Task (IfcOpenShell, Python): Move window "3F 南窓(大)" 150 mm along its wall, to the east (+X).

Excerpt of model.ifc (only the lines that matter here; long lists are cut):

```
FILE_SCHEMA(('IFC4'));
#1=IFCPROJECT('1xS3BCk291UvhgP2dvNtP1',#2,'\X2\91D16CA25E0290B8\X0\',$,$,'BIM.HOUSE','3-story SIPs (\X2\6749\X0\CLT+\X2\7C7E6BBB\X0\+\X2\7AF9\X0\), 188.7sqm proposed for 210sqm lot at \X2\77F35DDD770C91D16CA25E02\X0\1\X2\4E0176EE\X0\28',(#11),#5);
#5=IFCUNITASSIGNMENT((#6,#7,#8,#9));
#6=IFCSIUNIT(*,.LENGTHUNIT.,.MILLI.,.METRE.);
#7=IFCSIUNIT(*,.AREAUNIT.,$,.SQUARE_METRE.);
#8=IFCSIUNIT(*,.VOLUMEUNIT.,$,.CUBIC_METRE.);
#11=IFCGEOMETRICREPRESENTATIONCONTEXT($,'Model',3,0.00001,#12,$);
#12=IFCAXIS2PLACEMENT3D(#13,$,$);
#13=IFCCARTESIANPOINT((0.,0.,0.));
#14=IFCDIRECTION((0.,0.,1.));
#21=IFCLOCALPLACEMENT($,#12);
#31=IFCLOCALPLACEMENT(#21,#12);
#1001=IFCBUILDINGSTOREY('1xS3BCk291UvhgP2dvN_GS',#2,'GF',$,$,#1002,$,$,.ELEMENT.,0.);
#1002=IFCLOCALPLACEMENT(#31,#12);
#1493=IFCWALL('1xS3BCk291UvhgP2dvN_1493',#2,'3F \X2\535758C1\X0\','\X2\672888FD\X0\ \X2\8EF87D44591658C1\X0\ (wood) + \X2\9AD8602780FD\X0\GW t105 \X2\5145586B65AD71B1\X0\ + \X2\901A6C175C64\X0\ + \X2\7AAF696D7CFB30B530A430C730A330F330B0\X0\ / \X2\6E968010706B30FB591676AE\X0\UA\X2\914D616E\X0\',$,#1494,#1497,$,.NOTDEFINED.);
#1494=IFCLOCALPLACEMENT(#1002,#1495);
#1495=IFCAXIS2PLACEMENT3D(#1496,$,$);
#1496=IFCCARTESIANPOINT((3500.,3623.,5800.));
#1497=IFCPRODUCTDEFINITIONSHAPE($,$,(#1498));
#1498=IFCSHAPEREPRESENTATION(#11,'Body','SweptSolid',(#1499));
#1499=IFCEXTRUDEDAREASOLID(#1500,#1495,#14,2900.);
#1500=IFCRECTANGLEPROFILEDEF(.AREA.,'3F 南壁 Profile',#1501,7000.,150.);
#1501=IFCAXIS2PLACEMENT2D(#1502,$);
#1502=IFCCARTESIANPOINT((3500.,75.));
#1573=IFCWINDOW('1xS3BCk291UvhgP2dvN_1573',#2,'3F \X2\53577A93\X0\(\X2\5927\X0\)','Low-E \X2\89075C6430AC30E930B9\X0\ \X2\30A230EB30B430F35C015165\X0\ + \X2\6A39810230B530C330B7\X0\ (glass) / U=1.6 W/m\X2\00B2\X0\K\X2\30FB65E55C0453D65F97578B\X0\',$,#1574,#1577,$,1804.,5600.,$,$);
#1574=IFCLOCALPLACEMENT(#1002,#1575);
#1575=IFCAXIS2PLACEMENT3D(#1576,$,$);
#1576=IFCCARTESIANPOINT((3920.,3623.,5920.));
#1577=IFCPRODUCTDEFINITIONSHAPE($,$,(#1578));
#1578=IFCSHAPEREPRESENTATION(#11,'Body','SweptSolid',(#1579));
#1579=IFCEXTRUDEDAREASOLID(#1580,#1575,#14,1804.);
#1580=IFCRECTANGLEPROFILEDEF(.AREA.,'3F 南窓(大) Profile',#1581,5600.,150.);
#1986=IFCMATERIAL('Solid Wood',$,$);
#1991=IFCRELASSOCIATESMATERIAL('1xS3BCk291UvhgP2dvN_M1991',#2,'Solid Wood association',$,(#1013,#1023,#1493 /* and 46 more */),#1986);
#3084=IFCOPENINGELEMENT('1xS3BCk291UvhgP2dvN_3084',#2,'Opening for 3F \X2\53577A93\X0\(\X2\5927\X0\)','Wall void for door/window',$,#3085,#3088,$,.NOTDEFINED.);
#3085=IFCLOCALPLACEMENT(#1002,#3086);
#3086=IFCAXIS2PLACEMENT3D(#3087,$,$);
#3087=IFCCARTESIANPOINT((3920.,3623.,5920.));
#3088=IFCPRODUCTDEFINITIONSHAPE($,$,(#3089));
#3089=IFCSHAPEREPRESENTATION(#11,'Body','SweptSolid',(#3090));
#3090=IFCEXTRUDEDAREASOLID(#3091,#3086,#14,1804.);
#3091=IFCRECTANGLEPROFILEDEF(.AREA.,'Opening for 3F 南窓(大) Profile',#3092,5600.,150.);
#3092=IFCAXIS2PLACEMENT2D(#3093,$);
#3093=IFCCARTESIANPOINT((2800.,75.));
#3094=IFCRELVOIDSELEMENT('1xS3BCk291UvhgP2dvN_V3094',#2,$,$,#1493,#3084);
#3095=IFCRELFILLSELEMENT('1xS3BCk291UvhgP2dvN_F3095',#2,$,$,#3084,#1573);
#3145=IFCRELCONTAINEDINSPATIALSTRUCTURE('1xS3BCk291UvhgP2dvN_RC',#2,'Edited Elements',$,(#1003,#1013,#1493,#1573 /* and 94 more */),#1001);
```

```python
import ifcopenshell
import ifcopenshell.api.geometry
import ifcopenshell.util.placement

model = ifcopenshell.open("model.ifc")

window = model.by_guid("1xS3BCk291UvhgP2dvN_1573")
opening = window.FillsVoids[0].RelatingOpeningElement
wall = opening.VoidsElements[0].RelatingBuildingElement

wall_matrix = ifcopenshell.util.placement.get_local_placement(wall.ObjectPlacement)
shift = wall_matrix[:3, 0] * 150.0
before = ifcopenshell.util.placement.get_local_placement(window.ObjectPlacement)[:3, 3].copy()

# The window is not placed relative to its opening, so move both.
for product in (opening, window):
    matrix = ifcopenshell.util.placement.get_local_placement(product.ObjectPlacement)
    matrix[:3, 3] += shift
    ifcopenshell.api.geometry.edit_object_placement(model, product=product, matrix=matrix, is_si=False)

after = ifcopenshell.util.placement.get_local_placement(window.ObjectPlacement)[:3, 3]
print("window moved by", (after - before).round(3) + 0.0)

model.write("model_edited.ifc")
```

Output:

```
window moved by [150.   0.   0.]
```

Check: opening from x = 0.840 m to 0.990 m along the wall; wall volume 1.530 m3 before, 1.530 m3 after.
